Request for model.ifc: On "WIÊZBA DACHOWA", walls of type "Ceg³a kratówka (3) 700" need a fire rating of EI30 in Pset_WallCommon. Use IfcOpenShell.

First a look at what the model holds.

```python
import ifcopenshell
import ifcopenshell.util.element

model = ifcopenshell.open("model.ifc")
print(model.schema)
storey = next(s for s in model.by_type("IfcBuildingStorey") if s.Name == "WIÊZBA DACHOWA")
walls = [e for e in ifcopenshell.util.element.get_decomposition(storey) if e.is_a("IfcWall")]
seen = {}
for e in walls:
    element_type = ifcopenshell.util.element.get_type(e)
    key = (element_type.Name if element_type != e and element_type else None, ifcopenshell.util.element.get_pset(e, "Pset_WallCommon", "FireRating"))
    seen[key] = seen.get(key, 0) + 1
for (name, value), count in sorted(seen.items(), key=str):
    print(count, "x", name, "|", value)
```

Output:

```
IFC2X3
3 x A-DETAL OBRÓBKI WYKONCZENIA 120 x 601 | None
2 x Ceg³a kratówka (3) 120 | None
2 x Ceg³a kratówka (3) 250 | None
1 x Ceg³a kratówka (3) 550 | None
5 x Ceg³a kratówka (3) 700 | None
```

```python
import ifcopenshell
import ifcopenshell.api.pset
import ifcopenshell.util.element

model = ifcopenshell.open("model.ifc")

storey = next(s for s in model.by_type("IfcBuildingStorey") if s.Name == "WIÊZBA DACHOWA")
walls = [e for e in ifcopenshell.util.element.get_decomposition(storey) if e.is_a("IfcWall")]

count = 0
for e in walls:
    element_type = ifcopenshell.util.element.get_type(e)
    if element_type in (None, e) or element_type.Name != "Ceg³a kratówka (3) 700":
        continue
    # add_pset returns the element's existing set when there is one.
    pset = ifcopenshell.api.pset.add_pset(model, product=e, name="Pset_WallCommon")
    ifcopenshell.api.pset.edit_pset(model, pset=pset, properties={"FireRating": "EI30"})
    count += 1

print(count, "walls updated")

model.write("model_edited.ifc")
```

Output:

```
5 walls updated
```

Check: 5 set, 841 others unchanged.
